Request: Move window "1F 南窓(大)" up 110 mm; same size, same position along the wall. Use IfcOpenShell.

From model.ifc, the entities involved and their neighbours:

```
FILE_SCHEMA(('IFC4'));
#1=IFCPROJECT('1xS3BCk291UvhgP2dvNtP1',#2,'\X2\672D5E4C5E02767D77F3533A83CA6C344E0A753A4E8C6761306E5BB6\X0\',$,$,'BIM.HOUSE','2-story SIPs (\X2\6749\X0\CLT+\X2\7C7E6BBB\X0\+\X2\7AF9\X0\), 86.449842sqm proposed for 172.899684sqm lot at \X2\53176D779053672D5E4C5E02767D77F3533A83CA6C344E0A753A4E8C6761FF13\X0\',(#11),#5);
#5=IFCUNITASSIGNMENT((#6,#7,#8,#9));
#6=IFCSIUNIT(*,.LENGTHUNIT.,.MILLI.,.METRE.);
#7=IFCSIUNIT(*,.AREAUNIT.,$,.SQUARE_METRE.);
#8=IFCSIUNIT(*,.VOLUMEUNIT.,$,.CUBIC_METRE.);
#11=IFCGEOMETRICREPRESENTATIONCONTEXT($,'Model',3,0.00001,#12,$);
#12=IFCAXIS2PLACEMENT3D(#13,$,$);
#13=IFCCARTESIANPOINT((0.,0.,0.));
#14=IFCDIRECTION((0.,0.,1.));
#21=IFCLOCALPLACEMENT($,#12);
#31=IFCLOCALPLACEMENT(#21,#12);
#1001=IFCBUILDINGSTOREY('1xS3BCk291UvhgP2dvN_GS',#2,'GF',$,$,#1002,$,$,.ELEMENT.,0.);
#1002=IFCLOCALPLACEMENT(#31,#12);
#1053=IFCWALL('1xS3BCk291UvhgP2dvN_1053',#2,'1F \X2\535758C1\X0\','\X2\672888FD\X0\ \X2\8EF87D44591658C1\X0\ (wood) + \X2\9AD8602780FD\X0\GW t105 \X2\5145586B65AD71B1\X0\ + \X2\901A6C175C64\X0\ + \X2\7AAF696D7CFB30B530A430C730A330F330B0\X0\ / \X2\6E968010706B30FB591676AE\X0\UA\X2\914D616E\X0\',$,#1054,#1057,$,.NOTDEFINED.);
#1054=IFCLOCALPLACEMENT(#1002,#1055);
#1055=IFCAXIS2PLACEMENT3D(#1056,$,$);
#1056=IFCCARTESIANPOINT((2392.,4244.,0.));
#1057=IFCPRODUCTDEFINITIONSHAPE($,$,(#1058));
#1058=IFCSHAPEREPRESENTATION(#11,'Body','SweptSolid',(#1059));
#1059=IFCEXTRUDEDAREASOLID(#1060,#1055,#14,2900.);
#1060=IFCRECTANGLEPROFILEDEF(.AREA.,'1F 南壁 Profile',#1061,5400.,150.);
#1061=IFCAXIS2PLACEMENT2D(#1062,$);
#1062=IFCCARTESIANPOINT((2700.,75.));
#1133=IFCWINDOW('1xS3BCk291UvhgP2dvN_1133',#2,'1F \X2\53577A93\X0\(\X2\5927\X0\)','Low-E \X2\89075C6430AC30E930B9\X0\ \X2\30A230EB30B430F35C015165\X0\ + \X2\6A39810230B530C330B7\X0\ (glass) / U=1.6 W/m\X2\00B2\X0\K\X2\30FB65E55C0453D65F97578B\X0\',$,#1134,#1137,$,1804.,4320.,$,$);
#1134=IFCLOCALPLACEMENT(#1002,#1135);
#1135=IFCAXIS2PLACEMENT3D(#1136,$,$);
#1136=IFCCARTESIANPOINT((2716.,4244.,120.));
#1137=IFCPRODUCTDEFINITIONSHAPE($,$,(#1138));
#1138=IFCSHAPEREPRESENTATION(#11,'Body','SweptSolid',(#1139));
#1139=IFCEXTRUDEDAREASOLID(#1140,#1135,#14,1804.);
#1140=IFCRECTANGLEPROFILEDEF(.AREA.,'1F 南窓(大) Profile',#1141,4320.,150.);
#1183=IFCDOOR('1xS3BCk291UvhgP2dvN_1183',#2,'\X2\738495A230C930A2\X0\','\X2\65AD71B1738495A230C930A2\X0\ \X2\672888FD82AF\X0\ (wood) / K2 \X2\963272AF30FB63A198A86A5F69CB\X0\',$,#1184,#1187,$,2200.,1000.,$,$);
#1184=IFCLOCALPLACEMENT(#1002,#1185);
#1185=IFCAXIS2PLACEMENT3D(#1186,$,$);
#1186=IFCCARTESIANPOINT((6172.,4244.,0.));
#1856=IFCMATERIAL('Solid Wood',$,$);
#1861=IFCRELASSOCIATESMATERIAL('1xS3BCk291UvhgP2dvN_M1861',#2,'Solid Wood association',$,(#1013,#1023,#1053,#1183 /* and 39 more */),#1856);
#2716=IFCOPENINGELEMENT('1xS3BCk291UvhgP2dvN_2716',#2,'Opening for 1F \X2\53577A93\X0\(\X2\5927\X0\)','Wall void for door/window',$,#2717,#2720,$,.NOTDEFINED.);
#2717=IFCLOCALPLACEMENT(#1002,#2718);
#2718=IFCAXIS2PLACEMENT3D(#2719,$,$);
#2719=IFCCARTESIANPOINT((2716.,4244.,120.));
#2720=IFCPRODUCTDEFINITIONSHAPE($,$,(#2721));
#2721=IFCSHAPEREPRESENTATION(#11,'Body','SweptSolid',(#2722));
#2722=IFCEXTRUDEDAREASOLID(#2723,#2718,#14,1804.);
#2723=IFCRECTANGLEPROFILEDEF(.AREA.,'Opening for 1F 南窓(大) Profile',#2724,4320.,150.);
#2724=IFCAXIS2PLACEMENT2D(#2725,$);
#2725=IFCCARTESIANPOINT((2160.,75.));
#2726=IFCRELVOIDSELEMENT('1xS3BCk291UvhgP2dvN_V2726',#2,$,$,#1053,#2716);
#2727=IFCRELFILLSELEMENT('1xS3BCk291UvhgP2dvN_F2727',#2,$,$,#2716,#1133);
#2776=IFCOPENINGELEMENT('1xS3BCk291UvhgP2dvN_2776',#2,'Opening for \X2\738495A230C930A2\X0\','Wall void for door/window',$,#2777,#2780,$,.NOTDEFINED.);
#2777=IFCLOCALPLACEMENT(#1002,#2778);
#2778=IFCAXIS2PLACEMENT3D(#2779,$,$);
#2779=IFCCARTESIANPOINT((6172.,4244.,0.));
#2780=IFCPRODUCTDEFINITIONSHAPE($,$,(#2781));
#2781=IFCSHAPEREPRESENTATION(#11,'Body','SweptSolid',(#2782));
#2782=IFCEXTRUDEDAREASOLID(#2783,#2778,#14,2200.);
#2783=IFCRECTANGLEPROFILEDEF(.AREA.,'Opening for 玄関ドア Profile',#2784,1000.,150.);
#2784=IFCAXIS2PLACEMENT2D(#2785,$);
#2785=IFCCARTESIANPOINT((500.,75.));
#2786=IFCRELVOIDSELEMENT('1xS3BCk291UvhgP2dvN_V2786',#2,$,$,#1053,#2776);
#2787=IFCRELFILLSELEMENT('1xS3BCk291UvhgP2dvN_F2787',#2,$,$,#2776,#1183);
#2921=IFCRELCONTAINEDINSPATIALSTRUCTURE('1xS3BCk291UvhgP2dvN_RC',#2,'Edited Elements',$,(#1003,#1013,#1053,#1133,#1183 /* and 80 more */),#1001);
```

```python
import numpy as np
import ifcopenshell
import ifcopenshell.api.geometry
import ifcopenshell.util.placement
import ifcopenshell.util.unit

model = ifcopenshell.open("model.ifc")
unit_scale = ifcopenshell.util.unit.calculate_unit_scale(model)

window = model.by_id(1133)
opening = window.FillsVoids[0].RelatingOpeningElement
dz = 0.11 / unit_scale

shift = np.array([0.0, 0.0, dz])
# The window is not placed relative to its opening, so move both.
for product in (opening, window):
    matrix = ifcopenshell.util.placement.get_local_placement(product.ObjectPlacement)
    matrix[:3, 3] += shift
    ifcopenshell.api.geometry.edit_object_placement(model, product=product, matrix=matrix, is_si=False)

print(f"moved by {dz * unit_scale:+.3f} m")

model.write("model_rev.ifc")
```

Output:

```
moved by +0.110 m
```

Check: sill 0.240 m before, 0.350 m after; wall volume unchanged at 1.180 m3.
